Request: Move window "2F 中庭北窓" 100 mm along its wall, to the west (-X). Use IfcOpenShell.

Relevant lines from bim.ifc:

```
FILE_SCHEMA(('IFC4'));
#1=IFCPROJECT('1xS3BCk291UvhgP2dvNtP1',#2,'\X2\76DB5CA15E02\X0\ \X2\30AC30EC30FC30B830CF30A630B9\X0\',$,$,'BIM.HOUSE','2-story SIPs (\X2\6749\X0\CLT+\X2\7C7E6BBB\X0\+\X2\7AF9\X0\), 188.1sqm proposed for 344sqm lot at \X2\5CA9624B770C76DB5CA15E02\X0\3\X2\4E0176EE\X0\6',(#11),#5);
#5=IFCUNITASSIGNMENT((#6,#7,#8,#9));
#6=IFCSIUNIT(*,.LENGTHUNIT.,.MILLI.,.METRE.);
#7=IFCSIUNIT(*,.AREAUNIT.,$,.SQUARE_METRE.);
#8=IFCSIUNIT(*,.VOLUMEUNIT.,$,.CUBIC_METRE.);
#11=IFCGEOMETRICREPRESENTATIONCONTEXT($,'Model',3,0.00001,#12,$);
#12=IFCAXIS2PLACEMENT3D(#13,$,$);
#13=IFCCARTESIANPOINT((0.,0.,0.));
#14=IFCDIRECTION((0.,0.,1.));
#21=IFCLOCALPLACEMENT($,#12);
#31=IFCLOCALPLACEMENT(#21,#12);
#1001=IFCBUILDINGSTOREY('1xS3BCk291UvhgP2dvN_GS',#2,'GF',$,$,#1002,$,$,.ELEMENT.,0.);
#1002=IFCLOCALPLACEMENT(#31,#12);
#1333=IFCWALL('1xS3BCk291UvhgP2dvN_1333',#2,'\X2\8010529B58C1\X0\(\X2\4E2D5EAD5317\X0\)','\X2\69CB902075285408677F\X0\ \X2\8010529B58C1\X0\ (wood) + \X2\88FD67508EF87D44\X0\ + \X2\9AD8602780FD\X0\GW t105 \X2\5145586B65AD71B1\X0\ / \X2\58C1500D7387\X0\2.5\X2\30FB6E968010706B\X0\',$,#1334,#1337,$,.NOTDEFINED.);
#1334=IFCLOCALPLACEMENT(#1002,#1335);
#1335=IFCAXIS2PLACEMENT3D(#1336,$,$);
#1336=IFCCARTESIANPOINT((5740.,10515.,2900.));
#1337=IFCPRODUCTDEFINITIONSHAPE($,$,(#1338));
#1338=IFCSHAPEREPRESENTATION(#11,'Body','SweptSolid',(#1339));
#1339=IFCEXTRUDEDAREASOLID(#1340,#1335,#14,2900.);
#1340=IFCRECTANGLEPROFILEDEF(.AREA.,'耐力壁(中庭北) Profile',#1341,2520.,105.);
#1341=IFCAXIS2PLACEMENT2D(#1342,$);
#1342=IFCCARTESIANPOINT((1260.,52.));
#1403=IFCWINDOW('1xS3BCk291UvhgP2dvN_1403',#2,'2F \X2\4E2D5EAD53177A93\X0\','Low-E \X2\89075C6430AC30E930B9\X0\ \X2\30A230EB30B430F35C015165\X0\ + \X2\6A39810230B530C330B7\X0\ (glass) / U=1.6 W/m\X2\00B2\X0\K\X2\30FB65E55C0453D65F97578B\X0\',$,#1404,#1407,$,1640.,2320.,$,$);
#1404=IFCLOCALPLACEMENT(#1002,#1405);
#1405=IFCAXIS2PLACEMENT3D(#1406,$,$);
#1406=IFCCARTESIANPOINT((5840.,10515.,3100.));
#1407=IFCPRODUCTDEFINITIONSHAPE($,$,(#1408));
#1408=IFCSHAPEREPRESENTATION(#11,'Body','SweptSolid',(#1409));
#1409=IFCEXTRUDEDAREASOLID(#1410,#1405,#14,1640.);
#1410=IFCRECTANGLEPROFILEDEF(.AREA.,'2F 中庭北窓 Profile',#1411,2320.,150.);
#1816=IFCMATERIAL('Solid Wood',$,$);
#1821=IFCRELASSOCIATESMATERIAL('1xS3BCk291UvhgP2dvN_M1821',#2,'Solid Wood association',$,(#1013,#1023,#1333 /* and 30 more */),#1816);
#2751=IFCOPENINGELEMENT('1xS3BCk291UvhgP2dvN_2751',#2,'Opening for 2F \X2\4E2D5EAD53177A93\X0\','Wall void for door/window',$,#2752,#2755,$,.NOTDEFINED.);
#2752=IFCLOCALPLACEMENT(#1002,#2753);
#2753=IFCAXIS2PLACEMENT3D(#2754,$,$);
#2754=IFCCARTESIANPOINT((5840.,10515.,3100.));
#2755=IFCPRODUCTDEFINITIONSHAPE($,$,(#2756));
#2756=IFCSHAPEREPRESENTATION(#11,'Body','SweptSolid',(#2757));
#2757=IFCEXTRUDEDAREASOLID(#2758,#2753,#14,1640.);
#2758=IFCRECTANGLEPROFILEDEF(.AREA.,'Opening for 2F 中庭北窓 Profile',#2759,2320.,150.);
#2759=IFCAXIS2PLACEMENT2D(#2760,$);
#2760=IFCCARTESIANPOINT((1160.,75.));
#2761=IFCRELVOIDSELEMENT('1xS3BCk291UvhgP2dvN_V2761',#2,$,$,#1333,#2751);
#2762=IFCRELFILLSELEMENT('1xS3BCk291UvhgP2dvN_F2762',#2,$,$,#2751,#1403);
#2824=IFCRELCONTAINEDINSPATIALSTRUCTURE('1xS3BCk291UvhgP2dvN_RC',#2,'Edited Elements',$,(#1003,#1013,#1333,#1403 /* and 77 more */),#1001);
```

```python
import ifcopenshell
import ifcopenshell.api.geometry
import ifcopenshell.util.placement

model = ifcopenshell.open("bim.ifc")

window = model.by_id(1403)
opening = window.FillsVoids[0].RelatingOpeningElement
wall = opening.VoidsElements[0].RelatingBuildingElement

wall_matrix = ifcopenshell.util.placement.get_local_placement(wall.ObjectPlacement)
shift = wall_matrix[:3, 0] * -100.0
before = ifcopenshell.util.placement.get_local_placement(window.ObjectPlacement)[:3, 3].copy()

# The window is not placed relative to its opening, so move both.
for product in (opening, window):
    matrix = ifcopenshell.util.placement.get_local_placement(product.ObjectPlacement)
    matrix[:3, 3] += shift
    ifcopenshell.api.geometry.edit_object_placement(model, product=product, matrix=matrix, is_si=False)

after = ifcopenshell.util.placement.get_local_placement(window.ObjectPlacement)[:3, 3]
print("window moved by", (after - before).round(3) + 0.0)

model.write("bim_edited.ifc")
```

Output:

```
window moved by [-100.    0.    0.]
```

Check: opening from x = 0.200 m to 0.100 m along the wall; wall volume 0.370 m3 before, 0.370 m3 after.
